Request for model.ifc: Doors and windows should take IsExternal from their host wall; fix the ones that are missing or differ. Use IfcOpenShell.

First a look at what the model holds.

```python
import ifcopenshell
import ifcopenshell.util.element

model = ifcopenshell.open("model.ifc")
print(model.schema)
seen = {}
for e in model.by_type("IfcDoor") + model.by_type("IfcWindow"):
    if not e.FillsVoids:
        continue
    host = e.FillsVoids[0].RelatingOpeningElement.VoidsElements[0].RelatingBuildingElement
    own = ifcopenshell.util.element.get_pset(e, f"Pset_{e.is_a()[3:].removesuffix('StandardCase')}Common", "IsExternal")
    wall = ifcopenshell.util.element.get_pset(host, "Pset_WallCommon", "IsExternal")
    seen[e.is_a(), own, wall] = seen.get((e.is_a(), own, wall), 0) + 1
for (cls, own, wall), count in sorted(seen.items(), key=str):
    print(count, cls, "IsExternal:", own, "| host wall:", wall)
```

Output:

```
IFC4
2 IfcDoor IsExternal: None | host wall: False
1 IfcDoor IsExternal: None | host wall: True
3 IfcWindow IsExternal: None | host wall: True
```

```python
import ifcopenshell
import ifcopenshell.api.pset
import ifcopenshell.util.element

model = ifcopenshell.open("model.ifc")

count = 0
for ifc_class, pset_name in (("IfcDoor", "Pset_DoorCommon"), ("IfcWindow", "Pset_WindowCommon")):
    for e in model.by_type(ifc_class):
        if not e.FillsVoids:
            continue
        host = e.FillsVoids[0].RelatingOpeningElement.VoidsElements[0].RelatingBuildingElement
        external = ifcopenshell.util.element.get_pset(host, "Pset_WallCommon", "IsExternal")
        if external is None or ifcopenshell.util.element.get_pset(e, pset_name, "IsExternal") == external:
            continue
        pset = ifcopenshell.api.pset.add_pset(model, product=e, name=pset_name)
        ifcopenshell.api.pset.edit_pset(model, pset=pset, properties={"IsExternal": external})
        count += 1

print(count, "updated")

model.write("model_updated.ifc")
```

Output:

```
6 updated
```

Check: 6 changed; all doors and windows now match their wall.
